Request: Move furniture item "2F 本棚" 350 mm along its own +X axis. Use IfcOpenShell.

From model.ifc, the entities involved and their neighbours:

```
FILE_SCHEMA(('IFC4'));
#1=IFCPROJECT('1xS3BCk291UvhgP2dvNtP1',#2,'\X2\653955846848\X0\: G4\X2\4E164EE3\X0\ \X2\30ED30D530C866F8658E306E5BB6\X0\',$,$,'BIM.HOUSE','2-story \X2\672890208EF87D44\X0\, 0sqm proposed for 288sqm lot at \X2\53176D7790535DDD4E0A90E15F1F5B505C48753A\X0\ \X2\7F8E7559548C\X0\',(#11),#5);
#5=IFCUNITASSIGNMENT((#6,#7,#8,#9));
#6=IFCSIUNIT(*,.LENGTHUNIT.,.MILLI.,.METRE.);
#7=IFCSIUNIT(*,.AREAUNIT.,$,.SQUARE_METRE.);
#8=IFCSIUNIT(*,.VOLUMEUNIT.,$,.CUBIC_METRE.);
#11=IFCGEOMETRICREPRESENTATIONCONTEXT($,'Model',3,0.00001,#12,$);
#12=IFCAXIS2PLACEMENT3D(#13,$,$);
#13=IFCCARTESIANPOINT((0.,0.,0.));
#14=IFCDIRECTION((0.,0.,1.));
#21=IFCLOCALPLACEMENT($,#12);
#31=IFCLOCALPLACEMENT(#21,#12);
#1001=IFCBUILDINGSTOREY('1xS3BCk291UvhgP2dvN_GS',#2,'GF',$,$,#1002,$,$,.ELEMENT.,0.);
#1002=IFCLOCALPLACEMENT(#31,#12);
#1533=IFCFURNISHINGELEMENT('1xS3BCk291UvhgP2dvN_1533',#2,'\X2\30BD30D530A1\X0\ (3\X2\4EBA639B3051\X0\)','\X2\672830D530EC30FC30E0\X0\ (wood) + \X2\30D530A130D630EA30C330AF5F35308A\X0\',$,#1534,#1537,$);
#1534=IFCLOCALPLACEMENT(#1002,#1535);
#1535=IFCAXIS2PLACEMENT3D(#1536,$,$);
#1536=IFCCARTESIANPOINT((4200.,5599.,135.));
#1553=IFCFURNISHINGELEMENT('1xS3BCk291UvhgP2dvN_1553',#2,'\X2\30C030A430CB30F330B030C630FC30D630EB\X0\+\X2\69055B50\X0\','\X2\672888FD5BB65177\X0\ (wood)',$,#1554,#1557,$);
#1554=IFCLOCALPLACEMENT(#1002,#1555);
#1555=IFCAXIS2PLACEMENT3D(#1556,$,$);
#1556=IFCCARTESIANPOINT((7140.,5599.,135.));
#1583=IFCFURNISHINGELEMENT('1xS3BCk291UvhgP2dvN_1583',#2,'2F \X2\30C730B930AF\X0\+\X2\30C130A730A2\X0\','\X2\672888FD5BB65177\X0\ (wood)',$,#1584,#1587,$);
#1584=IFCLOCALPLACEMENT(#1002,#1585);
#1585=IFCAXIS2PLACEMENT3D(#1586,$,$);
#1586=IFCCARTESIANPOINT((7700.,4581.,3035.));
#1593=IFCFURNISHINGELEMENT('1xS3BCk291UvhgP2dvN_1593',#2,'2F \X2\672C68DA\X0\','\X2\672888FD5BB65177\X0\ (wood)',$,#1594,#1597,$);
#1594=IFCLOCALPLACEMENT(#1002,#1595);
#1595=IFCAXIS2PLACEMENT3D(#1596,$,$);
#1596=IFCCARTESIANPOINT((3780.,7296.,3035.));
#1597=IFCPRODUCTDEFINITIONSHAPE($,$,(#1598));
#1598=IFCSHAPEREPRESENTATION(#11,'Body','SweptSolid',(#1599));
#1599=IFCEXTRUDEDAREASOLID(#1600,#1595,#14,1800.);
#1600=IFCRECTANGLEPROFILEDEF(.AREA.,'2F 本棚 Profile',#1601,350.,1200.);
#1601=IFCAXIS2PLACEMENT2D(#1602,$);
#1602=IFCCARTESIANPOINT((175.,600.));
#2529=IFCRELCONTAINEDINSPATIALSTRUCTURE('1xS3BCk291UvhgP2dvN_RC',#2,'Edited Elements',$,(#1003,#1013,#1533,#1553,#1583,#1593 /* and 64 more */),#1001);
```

```python
import ifcopenshell
import ifcopenshell.api.geometry
import ifcopenshell.util.placement
import ifcopenshell.util.unit

model = ifcopenshell.open("model.ifc")
unit_scale = ifcopenshell.util.unit.calculate_unit_scale(model)

item = model.by_id(1593)
matrix = ifcopenshell.util.placement.get_local_placement(item.ObjectPlacement)
matrix[:3, 3] += matrix[:3, 0] * 0.35 / unit_scale
ifcopenshell.api.geometry.edit_object_placement(model, product=item, matrix=matrix, is_si=False)

print(ifcopenshell.util.placement.get_local_placement(item.ObjectPlacement).round(3) + 0.0)

model.write("model_updated.ifc")
```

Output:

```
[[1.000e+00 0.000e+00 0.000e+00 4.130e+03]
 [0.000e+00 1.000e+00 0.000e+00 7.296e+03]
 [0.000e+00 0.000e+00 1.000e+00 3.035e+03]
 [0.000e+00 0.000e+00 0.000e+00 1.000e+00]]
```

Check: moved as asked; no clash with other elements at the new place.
